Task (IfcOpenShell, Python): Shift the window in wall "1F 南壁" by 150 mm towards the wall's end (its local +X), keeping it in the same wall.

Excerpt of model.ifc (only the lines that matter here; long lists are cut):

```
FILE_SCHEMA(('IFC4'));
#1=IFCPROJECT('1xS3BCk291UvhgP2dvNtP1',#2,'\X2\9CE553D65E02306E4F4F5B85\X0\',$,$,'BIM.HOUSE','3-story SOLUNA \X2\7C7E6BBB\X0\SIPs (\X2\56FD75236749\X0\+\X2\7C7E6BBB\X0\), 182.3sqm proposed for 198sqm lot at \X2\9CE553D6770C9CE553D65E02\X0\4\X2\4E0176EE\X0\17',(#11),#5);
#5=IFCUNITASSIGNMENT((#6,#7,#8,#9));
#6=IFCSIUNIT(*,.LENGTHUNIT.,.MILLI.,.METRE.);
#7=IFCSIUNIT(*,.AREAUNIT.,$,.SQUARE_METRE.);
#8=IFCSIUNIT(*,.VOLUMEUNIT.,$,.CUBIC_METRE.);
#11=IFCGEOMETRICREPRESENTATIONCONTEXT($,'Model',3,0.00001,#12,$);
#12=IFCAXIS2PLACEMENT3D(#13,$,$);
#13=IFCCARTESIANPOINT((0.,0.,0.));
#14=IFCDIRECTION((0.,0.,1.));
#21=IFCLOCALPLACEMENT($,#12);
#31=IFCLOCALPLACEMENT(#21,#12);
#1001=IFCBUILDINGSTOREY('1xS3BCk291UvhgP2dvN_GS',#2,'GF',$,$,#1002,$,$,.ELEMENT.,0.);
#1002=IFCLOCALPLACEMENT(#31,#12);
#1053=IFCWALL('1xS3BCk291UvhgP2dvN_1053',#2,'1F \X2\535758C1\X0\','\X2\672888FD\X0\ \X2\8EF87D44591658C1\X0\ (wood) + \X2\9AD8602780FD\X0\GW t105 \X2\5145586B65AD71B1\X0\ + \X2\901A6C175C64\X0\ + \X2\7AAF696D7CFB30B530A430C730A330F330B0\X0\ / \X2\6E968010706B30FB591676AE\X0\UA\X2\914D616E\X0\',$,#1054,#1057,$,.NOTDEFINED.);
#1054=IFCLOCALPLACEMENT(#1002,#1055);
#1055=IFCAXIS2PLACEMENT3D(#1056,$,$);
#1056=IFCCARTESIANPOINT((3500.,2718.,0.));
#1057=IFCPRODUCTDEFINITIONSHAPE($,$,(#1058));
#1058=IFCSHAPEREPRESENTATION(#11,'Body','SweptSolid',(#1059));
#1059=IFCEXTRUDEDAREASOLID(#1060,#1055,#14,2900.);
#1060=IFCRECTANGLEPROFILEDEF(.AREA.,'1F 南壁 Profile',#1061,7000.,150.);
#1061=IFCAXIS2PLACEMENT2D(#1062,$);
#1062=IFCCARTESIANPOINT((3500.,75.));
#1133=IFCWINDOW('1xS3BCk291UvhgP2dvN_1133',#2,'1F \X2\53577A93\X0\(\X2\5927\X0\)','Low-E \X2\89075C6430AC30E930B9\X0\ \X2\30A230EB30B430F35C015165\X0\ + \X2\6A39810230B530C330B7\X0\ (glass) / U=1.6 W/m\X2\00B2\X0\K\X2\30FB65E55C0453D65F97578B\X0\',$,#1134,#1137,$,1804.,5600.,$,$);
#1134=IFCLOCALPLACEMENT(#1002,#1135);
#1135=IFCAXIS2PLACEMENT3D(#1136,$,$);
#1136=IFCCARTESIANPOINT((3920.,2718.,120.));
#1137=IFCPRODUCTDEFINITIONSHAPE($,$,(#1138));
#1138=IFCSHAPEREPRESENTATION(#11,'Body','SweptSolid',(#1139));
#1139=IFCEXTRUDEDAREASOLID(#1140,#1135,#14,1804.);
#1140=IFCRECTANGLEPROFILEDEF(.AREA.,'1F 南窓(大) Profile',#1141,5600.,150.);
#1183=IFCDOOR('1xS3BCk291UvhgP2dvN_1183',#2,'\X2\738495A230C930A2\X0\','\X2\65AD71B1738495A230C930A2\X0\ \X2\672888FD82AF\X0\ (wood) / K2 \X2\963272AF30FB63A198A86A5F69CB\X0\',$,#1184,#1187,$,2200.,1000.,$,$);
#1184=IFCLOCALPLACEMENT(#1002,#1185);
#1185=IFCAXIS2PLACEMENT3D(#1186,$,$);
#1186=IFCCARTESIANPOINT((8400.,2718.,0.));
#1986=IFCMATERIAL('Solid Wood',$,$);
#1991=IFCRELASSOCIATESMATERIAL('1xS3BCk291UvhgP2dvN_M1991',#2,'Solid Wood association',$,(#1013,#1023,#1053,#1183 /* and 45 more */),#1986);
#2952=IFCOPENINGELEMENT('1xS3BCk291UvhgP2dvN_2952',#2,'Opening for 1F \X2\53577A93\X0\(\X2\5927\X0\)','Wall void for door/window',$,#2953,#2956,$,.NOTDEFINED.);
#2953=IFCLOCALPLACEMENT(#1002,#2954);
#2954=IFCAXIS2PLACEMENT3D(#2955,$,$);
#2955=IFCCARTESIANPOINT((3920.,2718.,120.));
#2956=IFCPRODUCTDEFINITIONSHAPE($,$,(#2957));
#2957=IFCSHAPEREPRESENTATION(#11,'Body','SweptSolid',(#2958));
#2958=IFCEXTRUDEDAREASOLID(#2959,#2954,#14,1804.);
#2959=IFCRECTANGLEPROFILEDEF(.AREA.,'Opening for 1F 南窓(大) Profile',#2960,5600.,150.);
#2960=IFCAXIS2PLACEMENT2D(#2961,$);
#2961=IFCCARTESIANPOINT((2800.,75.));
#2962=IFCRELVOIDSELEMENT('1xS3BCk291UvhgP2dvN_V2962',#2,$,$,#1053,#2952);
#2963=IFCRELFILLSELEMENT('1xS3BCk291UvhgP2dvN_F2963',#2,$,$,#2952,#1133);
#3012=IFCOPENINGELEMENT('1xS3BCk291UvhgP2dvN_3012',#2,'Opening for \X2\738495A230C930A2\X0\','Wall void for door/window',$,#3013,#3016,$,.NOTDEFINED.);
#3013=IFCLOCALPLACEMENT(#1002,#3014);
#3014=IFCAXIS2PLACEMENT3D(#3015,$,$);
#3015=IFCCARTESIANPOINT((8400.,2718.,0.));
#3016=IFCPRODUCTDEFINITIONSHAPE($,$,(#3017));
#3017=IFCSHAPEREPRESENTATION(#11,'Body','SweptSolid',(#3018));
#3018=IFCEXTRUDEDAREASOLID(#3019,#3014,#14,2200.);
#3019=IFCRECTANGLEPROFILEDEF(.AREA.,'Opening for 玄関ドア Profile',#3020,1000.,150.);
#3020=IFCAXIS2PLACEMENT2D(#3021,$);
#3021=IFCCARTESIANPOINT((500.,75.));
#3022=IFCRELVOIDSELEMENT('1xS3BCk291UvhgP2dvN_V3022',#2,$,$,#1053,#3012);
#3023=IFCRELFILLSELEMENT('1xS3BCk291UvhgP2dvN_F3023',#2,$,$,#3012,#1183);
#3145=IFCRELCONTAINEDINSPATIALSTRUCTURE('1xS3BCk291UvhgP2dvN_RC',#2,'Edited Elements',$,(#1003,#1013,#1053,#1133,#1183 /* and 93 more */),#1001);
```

```python
import ifcopenshell
import ifcopenshell.api.geometry
import ifcopenshell.util.placement
import ifcopenshell.util.unit

model = ifcopenshell.open("model.ifc")
unit_scale = ifcopenshell.util.unit.calculate_unit_scale(model)

window = model.by_guid("1xS3BCk291UvhgP2dvN_1133")
opening = window.FillsVoids[0].RelatingOpeningElement
wall = opening.VoidsElements[0].RelatingBuildingElement

wall_matrix = ifcopenshell.util.placement.get_local_placement(wall.ObjectPlacement)
shift = wall_matrix[:3, 0] * 0.15 / unit_scale
before = ifcopenshell.util.placement.get_local_placement(window.ObjectPlacement)[:3, 3].copy()

# The window is not placed relative to its opening, so move both.
for product in (opening, window):
    matrix = ifcopenshell.util.placement.get_local_placement(product.ObjectPlacement)
    matrix[:3, 3] += shift
    ifcopenshell.api.geometry.edit_object_placement(model, product=product, matrix=matrix, is_si=False)

after = ifcopenshell.util.placement.get_local_placement(window.ObjectPlacement)[:3, 3]
print("window moved by", (after - before).round(3) + 0.0)

model.write("model_updated.ifc")
```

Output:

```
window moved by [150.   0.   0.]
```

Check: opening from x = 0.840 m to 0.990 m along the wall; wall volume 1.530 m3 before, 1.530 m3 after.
